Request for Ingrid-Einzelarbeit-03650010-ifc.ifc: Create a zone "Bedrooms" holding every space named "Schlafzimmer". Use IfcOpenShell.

First a look at what the model holds.

```python
import ifcopenshell

model = ifcopenshell.open("Ingrid-Einzelarbeit-03650010-ifc.ifc")
print(model.schema)
seen = {}
for space in model.by_type("IfcSpace"):
    seen[space.LongName] = seen.get(space.LongName, 0) + 1
for name, count in sorted(seen.items(), key=str):
    print(count, "x", name)
print("zones:", [z.Name for z in model.by_type("IfcZone")][:20])
```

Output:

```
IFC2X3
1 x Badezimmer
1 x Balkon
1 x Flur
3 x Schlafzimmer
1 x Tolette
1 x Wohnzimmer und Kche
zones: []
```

```python
import ifcopenshell
import ifcopenshell.api.group
import ifcopenshell.api.root

model = ifcopenshell.open("Ingrid-Einzelarbeit-03650010-ifc.ifc")

names = {"Schlafzimmer"}
spaces = [s for s in model.by_type("IfcSpace") if s.LongName in names]

zone = ifcopenshell.api.root.create_entity(model, ifc_class="IfcZone", name="Bedrooms")
ifcopenshell.api.group.assign_group(model, products=spaces, group=zone)
print(len(spaces), "spaces in", zone.Name)

model.write("Ingrid-Einzelarbeit-03650010-ifc-out.ifc")
```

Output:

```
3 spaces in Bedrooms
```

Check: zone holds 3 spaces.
